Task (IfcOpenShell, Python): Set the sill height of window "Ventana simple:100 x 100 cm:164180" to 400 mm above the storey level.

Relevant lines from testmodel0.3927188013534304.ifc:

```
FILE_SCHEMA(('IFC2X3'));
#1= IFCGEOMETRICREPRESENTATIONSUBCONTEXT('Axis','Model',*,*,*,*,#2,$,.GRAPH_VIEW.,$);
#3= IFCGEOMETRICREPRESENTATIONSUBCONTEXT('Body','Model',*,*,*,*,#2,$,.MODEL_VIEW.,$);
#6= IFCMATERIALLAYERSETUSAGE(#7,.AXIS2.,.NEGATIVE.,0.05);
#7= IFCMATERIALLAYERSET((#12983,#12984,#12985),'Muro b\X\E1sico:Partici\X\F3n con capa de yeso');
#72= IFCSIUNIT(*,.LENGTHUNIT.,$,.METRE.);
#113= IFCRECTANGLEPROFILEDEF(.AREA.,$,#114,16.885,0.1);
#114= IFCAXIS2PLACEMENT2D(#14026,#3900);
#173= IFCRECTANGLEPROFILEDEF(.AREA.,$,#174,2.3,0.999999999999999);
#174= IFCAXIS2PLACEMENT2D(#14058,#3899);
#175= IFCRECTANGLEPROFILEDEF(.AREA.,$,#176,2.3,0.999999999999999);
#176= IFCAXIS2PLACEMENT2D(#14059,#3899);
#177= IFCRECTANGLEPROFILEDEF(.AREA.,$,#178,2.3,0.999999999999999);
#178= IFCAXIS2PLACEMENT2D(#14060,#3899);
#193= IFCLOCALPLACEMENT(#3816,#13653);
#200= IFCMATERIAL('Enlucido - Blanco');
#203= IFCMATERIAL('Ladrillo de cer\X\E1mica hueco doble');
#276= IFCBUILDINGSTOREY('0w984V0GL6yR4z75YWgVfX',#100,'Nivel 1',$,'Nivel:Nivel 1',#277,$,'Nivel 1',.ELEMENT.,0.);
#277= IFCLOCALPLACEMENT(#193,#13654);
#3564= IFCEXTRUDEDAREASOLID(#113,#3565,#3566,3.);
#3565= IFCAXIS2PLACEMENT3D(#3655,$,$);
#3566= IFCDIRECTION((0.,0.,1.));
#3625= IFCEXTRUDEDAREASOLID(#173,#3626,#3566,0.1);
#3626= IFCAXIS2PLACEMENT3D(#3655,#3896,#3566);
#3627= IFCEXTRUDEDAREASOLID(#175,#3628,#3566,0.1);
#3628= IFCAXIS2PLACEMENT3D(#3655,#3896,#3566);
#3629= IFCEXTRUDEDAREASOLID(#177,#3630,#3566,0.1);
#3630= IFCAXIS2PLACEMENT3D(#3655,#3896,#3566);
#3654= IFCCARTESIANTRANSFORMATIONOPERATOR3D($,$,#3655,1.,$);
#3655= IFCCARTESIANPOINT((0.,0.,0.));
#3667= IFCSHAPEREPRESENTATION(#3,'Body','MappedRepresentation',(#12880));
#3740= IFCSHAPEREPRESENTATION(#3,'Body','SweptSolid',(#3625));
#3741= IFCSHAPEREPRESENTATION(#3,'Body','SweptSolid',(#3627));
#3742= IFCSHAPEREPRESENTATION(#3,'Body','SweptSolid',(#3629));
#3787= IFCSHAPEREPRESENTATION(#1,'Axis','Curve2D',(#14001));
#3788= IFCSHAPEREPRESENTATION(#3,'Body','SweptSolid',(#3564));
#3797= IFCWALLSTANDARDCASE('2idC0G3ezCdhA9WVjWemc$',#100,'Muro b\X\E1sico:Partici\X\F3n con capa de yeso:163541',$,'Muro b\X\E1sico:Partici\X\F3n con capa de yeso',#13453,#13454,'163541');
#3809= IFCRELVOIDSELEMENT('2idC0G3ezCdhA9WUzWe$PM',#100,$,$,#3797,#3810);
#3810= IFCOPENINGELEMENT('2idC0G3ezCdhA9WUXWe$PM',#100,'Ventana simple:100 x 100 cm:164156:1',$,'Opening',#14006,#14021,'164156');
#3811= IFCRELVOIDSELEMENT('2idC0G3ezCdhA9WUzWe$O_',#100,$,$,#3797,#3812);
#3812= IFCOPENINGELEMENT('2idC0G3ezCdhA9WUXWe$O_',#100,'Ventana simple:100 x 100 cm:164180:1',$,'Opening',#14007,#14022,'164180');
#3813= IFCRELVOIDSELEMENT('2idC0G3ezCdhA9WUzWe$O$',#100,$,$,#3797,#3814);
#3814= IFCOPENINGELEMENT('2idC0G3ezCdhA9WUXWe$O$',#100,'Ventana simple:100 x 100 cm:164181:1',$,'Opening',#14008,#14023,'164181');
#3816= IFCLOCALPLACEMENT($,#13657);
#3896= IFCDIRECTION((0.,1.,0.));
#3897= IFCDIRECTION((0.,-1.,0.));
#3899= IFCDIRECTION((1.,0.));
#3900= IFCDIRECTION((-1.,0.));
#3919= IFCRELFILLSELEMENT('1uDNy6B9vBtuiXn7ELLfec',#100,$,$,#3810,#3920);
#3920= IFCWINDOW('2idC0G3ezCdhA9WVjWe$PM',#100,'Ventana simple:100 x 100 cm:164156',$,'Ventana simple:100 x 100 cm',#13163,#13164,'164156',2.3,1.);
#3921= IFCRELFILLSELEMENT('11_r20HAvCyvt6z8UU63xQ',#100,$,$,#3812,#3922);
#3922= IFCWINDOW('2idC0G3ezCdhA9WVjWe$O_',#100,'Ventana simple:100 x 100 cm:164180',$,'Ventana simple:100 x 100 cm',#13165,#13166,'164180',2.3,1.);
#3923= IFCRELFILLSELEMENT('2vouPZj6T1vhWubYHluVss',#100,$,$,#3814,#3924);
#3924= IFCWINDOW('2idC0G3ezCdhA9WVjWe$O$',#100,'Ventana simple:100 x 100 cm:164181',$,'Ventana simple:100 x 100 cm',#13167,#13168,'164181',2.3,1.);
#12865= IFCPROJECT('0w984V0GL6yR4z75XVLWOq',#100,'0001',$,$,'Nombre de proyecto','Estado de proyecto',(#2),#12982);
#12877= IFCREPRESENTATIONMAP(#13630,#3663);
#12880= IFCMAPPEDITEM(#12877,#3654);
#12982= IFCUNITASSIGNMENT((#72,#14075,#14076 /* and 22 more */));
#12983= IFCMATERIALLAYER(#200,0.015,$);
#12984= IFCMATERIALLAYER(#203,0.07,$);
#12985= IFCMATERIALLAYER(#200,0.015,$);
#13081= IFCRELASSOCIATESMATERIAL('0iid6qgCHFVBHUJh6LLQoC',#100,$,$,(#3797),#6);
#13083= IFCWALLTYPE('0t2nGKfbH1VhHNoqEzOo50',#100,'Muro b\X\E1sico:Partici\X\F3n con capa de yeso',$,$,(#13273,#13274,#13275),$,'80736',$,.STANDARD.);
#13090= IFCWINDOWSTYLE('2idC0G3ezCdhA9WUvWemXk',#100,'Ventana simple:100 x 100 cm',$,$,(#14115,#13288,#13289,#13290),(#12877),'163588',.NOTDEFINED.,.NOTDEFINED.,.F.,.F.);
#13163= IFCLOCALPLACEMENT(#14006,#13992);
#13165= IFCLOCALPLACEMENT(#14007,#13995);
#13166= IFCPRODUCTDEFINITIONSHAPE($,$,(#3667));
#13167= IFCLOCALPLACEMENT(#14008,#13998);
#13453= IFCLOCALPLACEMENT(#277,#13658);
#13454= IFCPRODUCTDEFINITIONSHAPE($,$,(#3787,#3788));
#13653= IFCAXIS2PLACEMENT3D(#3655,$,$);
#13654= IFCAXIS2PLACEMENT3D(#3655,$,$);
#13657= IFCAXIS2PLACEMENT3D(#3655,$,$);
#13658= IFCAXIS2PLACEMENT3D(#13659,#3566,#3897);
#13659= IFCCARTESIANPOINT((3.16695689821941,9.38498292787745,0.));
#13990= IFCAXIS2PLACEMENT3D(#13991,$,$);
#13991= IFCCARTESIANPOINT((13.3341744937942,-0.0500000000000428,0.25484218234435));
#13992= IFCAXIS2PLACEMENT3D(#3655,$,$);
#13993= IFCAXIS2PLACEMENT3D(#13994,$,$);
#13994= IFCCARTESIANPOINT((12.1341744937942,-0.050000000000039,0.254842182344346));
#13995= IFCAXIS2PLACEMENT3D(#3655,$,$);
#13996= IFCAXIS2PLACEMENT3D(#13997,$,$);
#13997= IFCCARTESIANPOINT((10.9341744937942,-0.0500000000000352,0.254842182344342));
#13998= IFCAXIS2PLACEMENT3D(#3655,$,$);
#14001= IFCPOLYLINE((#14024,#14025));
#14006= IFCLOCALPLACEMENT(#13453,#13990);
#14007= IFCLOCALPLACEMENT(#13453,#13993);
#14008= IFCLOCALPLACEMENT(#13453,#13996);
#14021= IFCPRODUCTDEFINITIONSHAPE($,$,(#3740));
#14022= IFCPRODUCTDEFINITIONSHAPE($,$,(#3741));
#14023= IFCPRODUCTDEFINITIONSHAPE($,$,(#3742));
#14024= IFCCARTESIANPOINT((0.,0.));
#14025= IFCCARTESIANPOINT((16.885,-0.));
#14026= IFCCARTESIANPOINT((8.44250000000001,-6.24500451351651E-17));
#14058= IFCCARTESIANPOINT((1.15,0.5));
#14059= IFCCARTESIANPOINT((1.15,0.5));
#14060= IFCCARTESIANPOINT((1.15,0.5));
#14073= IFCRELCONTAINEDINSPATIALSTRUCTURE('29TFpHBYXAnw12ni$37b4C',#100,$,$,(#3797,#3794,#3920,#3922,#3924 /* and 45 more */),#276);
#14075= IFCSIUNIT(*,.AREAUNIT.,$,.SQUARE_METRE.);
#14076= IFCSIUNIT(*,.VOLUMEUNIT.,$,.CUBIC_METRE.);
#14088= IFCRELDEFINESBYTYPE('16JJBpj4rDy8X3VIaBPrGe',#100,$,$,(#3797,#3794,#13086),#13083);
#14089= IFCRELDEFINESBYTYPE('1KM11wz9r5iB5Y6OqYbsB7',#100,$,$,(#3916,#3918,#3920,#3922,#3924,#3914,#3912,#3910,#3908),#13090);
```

```python
import numpy as np
import ifcopenshell
import ifcopenshell.api.geometry
import ifcopenshell.geom
import ifcopenshell.util.element
import ifcopenshell.util.placement
import ifcopenshell.util.shape
import ifcopenshell.util.unit

model = ifcopenshell.open("testmodel0.3927188013534304.ifc")
unit_scale = ifcopenshell.util.unit.calculate_unit_scale(model)

window = model.by_guid("2idC0G3ezCdhA9WVjWe$O_")
opening = window.FillsVoids[0].RelatingOpeningElement
storey = ifcopenshell.util.element.get_container(window, ifc_class="IfcBuildingStorey")
level = ifcopenshell.util.placement.get_local_placement(storey.ObjectPlacement)[2, 3]

# The opening's origin need not be at the sill, so measure its lowest point.
shape = ifcopenshell.geom.create_shape(ifcopenshell.geom.settings(), opening)
bottom = ifcopenshell.util.shape.get_shape_bottom_elevation(shape, shape.geometry) / unit_scale
dz = level + 0.4 / unit_scale - bottom

shift = np.array([0.0, 0.0, dz])
# The window is placed relative to its opening, so it follows when the opening moves.
matrix = ifcopenshell.util.placement.get_local_placement(opening.ObjectPlacement)
matrix[:3, 3] += shift
ifcopenshell.api.geometry.edit_object_placement(
    model, product=opening, matrix=matrix, is_si=False, should_transform_children=True
)

print(f"moved by {dz * unit_scale:+.3f} m")

model.write("testmodel0.3927188013534304_updated.ifc")
```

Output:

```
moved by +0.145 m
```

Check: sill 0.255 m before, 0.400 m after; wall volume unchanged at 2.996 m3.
